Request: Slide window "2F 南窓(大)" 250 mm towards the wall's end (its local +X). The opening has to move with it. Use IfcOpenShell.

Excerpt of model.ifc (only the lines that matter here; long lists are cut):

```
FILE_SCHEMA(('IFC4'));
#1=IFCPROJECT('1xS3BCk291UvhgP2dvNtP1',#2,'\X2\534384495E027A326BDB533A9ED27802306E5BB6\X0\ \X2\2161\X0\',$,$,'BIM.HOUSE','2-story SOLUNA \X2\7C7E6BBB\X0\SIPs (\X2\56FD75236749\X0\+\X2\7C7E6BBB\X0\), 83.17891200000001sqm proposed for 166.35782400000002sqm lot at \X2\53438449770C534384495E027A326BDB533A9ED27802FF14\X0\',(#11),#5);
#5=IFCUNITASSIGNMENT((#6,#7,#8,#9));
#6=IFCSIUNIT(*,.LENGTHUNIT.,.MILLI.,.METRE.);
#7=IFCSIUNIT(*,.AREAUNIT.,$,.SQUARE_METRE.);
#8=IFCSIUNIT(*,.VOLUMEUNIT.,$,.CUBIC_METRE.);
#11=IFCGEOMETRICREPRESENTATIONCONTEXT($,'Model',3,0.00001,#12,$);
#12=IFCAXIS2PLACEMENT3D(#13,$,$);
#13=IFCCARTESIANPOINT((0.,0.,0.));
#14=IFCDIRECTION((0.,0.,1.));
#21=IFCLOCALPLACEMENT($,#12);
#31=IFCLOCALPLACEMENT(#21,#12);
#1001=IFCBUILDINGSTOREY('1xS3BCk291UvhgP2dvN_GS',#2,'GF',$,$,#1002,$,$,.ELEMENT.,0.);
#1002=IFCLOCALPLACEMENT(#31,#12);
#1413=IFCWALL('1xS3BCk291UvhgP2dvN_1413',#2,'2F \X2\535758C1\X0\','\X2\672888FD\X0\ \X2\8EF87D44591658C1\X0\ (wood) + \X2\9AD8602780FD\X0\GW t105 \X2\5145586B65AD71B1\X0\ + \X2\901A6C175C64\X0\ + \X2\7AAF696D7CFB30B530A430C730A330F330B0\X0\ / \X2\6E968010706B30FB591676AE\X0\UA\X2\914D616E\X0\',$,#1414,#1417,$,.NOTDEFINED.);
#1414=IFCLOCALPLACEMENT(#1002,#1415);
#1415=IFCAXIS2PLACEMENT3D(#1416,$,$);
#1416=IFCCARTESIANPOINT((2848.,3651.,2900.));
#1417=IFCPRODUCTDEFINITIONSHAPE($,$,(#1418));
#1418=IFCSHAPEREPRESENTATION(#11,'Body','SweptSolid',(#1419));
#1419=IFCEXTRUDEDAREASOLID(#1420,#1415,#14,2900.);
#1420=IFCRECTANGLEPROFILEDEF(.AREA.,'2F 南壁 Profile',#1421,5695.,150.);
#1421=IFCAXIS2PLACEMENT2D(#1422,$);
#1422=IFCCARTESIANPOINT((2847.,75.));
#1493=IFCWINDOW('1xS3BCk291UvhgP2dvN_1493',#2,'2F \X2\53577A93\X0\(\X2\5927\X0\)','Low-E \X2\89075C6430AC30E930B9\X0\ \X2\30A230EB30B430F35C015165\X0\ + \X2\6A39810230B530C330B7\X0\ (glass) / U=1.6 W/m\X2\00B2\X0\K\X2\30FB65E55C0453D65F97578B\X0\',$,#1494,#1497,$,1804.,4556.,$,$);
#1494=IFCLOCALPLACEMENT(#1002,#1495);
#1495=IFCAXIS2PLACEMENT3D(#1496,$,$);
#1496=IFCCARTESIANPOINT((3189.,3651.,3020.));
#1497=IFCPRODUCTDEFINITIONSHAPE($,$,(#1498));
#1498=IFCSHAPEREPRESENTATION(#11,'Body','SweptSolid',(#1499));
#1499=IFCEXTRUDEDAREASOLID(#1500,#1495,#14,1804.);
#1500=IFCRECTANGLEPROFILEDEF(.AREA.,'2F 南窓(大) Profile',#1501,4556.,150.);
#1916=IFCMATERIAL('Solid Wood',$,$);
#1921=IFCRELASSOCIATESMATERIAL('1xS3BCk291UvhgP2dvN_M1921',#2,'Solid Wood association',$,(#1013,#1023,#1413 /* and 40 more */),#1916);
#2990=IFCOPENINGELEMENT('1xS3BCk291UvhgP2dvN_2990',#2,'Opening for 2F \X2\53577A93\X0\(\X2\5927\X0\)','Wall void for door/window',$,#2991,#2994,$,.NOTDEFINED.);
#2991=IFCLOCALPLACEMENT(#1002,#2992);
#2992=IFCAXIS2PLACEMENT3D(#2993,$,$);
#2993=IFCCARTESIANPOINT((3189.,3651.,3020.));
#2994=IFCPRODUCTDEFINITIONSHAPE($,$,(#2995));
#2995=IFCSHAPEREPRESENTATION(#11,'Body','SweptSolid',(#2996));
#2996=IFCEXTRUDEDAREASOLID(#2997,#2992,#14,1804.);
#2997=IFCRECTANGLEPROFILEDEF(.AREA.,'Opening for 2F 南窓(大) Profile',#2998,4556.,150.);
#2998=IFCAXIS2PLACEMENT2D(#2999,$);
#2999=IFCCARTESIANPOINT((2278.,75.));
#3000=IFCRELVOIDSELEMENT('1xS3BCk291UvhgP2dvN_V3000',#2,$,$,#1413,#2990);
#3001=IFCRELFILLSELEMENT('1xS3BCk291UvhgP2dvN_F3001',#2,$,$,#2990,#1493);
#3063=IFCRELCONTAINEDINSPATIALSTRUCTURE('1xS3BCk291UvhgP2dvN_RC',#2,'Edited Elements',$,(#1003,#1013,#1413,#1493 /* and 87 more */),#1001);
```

```python
import ifcopenshell
import ifcopenshell.api.geometry
import ifcopenshell.util.placement
import ifcopenshell.util.unit

model = ifcopenshell.open("model.ifc")
unit_scale = ifcopenshell.util.unit.calculate_unit_scale(model)

window = model.by_guid("1xS3BCk291UvhgP2dvN_1493")
opening = window.FillsVoids[0].RelatingOpeningElement
wall = opening.VoidsElements[0].RelatingBuildingElement

wall_matrix = ifcopenshell.util.placement.get_local_placement(wall.ObjectPlacement)
shift = wall_matrix[:3, 0] * 0.25 / unit_scale
before = ifcopenshell.util.placement.get_local_placement(window.ObjectPlacement)[:3, 3].copy()

# The window is not placed relative to its opening, so move both.
for product in (opening, window):
    matrix = ifcopenshell.util.placement.get_local_placement(product.ObjectPlacement)
    matrix[:3, 3] += shift
    ifcopenshell.api.geometry.edit_object_placement(model, product=product, matrix=matrix, is_si=False)

after = ifcopenshell.util.placement.get_local_placement(window.ObjectPlacement)[:3, 3]
print("window moved by", (after - before).round(3) + 0.0)

model.write("model-out.ifc")
```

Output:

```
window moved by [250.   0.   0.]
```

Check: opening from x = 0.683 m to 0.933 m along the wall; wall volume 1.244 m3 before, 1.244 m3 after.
